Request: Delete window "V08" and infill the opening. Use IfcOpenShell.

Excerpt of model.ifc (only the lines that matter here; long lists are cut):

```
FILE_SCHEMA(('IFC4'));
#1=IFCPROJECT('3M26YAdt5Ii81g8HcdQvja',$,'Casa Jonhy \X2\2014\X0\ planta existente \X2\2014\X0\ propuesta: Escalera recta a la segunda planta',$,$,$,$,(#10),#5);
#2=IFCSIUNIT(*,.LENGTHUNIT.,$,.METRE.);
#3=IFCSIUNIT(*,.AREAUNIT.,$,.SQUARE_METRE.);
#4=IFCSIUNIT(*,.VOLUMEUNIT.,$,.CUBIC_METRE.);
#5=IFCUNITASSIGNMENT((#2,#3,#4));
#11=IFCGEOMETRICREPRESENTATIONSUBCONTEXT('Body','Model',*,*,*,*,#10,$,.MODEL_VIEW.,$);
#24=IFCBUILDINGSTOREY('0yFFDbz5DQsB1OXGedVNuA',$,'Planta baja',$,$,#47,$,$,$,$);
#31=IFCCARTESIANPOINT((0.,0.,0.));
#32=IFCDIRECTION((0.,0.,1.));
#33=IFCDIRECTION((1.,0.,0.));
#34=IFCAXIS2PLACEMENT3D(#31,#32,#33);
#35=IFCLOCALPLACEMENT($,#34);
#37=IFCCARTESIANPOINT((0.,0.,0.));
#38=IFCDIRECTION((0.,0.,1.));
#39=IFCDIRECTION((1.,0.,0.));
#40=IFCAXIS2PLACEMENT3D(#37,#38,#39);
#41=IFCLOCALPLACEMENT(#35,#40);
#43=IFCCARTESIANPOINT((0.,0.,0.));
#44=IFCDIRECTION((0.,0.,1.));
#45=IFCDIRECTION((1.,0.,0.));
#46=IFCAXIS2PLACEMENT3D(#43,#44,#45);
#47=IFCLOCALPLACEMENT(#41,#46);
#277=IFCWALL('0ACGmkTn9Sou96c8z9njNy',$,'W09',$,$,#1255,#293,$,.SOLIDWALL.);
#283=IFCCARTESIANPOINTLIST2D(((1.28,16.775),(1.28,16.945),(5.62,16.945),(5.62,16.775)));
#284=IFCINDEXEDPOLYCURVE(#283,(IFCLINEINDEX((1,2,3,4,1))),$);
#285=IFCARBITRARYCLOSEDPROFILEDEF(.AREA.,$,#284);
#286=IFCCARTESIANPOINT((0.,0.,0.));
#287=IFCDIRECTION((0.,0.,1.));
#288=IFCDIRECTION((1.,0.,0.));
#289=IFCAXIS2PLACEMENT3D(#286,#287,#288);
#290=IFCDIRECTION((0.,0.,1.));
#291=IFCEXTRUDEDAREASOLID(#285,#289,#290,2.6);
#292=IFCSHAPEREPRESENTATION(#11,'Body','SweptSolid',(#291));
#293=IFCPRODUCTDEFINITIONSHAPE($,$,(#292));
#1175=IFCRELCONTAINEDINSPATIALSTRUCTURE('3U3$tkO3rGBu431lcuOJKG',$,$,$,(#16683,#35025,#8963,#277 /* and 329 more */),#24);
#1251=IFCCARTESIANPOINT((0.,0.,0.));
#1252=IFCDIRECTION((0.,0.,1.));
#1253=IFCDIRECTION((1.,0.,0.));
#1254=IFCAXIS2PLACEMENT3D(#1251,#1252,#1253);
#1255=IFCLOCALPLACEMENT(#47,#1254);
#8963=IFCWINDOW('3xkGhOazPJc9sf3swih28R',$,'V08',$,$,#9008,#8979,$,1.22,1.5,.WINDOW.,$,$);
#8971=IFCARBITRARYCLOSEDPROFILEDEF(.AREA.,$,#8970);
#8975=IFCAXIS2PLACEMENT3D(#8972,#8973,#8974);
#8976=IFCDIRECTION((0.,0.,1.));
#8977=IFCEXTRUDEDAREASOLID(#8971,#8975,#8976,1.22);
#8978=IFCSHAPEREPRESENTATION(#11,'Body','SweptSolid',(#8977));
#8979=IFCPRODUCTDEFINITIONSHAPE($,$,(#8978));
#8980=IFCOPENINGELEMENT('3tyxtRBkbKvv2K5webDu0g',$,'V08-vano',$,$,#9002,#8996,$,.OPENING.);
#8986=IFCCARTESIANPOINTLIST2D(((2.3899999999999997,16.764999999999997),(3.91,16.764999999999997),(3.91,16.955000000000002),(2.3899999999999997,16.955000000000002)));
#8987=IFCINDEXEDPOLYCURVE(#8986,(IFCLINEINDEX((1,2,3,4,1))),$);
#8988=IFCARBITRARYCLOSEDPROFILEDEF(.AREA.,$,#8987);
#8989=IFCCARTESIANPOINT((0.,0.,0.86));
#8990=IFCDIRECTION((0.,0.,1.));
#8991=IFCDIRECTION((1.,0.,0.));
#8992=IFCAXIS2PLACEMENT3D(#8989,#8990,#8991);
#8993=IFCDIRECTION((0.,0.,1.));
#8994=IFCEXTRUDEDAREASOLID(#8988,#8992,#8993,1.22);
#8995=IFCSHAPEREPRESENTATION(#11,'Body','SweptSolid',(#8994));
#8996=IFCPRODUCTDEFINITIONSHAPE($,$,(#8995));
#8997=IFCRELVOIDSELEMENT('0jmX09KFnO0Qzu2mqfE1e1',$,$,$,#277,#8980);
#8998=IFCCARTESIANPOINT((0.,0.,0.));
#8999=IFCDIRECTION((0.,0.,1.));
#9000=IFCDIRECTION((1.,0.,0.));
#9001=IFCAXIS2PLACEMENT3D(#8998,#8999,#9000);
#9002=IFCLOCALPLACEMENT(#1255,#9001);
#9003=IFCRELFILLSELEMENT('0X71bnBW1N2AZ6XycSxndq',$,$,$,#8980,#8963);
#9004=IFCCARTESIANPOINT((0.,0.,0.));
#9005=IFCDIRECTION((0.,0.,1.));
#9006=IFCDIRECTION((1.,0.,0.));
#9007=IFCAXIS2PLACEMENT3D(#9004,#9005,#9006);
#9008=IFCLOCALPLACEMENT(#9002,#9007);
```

```python
import ifcopenshell
import ifcopenshell.api.feature
import ifcopenshell.api.root
import ifcopenshell.geom
import ifcopenshell.util.shape

model = ifcopenshell.open("model.ifc")
settings = ifcopenshell.geom.settings()


def volume(element):
    """Net volume in cubic metres, openings subtracted."""
    shape = ifcopenshell.geom.create_shape(settings, element)
    return ifcopenshell.util.shape.get_volume(shape.geometry)


window = model.by_guid("3xkGhOazPJc9sf3swih28R")
opening = window.FillsVoids[0].RelatingOpeningElement
wall = opening.VoidsElements[0].RelatingBuildingElement
before = volume(wall)

ifcopenshell.api.root.remove_product(model, product=window)
ifcopenshell.api.feature.remove_feature(model, feature=opening)

after = volume(wall)

print(f"wall volume {before:.3f} -> {after:.3f} m3")

model.write("model_rev.ifc")
```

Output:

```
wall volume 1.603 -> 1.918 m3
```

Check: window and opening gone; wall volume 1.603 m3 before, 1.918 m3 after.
